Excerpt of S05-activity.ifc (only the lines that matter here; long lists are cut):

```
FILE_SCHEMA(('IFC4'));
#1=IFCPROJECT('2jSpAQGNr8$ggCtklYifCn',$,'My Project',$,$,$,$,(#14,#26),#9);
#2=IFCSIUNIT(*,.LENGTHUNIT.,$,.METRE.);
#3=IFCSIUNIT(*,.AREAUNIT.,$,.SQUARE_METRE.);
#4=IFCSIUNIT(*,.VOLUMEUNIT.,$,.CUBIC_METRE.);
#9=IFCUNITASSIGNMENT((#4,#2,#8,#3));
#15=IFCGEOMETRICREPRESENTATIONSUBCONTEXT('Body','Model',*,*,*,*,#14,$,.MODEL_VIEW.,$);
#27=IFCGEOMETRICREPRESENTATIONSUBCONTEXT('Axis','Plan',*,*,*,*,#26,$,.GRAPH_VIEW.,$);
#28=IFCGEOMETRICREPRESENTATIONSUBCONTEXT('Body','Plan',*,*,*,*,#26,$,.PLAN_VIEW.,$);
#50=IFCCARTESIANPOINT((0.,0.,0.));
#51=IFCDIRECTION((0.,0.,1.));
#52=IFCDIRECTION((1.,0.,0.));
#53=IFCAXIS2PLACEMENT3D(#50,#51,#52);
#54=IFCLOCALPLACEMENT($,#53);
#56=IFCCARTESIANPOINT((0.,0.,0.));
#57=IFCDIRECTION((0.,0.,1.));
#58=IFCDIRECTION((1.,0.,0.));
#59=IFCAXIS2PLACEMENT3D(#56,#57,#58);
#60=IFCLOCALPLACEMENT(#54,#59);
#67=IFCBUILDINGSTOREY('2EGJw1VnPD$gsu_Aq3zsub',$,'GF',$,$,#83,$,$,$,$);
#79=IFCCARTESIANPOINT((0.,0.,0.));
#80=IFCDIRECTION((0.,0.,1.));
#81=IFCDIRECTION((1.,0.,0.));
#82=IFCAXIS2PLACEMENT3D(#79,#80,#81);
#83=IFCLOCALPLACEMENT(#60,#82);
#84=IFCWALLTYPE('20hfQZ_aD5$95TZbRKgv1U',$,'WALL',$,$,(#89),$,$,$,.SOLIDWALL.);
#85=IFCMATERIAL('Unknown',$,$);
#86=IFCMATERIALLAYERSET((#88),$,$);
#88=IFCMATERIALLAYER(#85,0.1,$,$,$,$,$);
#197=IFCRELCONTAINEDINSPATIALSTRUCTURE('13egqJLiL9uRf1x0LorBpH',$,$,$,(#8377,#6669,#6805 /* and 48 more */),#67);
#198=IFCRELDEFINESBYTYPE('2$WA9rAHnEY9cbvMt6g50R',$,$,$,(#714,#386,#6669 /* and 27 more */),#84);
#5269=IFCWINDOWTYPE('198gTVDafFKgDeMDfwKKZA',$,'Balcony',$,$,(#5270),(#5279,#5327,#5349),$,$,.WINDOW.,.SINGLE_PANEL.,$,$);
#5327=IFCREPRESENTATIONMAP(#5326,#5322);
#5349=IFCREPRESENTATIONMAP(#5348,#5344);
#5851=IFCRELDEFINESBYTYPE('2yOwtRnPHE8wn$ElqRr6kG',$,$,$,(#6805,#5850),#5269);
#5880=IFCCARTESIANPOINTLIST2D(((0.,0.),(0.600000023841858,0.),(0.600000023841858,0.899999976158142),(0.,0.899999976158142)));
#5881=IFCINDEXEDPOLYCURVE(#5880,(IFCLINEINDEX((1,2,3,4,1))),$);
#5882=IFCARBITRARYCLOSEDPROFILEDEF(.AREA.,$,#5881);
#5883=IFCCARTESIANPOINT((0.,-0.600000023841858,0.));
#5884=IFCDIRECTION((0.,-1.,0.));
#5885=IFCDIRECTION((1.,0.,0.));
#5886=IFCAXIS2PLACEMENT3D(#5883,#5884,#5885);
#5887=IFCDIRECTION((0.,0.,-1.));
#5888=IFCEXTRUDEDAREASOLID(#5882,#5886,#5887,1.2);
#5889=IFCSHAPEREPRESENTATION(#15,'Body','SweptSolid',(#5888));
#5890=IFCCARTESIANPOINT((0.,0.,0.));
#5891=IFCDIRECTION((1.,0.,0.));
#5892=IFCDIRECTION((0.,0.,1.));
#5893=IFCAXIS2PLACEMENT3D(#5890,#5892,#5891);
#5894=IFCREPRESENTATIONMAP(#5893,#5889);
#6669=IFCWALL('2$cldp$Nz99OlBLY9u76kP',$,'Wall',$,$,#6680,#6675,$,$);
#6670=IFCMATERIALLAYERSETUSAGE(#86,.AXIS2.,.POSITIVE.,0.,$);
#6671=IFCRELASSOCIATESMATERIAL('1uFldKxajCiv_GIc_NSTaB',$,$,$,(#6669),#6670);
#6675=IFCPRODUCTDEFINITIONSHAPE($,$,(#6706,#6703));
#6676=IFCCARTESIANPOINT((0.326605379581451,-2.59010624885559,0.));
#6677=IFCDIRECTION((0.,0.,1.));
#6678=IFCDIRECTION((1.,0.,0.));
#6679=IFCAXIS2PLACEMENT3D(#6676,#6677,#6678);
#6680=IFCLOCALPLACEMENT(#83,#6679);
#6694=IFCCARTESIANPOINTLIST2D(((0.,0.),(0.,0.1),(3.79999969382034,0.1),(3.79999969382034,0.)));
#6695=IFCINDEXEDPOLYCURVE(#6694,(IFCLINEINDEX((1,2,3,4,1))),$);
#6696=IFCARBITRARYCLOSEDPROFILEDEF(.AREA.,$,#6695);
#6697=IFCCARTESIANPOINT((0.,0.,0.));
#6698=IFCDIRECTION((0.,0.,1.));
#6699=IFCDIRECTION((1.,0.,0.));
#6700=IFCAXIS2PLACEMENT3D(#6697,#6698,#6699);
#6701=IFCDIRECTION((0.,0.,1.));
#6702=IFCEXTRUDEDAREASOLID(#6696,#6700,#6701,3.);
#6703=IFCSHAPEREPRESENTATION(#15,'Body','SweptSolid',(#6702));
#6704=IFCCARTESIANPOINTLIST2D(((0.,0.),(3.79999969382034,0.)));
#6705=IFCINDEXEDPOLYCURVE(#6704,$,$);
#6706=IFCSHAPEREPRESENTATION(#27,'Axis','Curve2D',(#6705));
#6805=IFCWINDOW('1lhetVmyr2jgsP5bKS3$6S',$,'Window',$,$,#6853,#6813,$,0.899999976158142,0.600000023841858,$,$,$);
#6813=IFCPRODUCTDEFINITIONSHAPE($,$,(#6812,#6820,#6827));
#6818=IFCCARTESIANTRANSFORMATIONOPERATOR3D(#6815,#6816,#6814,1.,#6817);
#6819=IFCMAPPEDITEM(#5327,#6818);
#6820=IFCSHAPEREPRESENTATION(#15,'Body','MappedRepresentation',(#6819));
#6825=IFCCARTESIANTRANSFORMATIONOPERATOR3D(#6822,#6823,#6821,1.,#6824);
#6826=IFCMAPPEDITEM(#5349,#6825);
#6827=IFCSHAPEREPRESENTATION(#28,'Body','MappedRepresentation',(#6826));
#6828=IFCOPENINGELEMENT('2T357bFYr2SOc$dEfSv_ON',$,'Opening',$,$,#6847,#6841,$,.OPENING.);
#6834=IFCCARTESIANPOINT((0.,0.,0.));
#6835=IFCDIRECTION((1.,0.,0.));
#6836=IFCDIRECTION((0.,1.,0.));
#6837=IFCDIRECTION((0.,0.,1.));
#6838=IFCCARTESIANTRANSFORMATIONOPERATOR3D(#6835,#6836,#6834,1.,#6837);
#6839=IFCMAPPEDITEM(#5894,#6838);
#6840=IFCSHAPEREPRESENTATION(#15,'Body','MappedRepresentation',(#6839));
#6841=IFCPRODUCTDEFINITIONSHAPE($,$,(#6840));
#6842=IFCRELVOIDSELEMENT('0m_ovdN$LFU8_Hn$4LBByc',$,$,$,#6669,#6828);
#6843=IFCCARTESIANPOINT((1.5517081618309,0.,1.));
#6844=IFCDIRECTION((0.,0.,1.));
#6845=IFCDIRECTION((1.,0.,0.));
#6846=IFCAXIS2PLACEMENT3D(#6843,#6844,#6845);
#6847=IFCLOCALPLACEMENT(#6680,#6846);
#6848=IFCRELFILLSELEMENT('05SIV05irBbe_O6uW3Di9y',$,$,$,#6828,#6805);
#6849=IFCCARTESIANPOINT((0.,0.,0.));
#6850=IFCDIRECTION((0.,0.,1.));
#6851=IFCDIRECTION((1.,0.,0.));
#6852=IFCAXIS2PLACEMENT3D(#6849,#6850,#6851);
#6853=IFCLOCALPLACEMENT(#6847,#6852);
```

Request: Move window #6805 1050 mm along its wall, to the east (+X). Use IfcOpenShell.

```python
import ifcopenshell
import ifcopenshell.api.geometry
import ifcopenshell.util.placement

model = ifcopenshell.open("S05-activity.ifc")

window = model.by_guid("1lhetVmyr2jgsP5bKS3$6S")
opening = window.FillsVoids[0].RelatingOpeningElement
wall = opening.VoidsElements[0].RelatingBuildingElement

wall_matrix = ifcopenshell.util.placement.get_local_placement(wall.ObjectPlacement)
shift = wall_matrix[:3, 0] * 1.05
before = ifcopenshell.util.placement.get_local_placement(window.ObjectPlacement)[:3, 3].copy()

# The window is placed relative to its opening, so it follows when the opening moves.
matrix = ifcopenshell.util.placement.get_local_placement(opening.ObjectPlacement)
matrix[:3, 3] += shift
ifcopenshell.api.geometry.edit_object_placement(
    model, product=opening, matrix=matrix, is_si=False, should_transform_children=True
)

after = ifcopenshell.util.placement.get_local_placement(window.ObjectPlacement)[:3, 3]
print("window moved by", (after - before).round(3) + 0.0)

model.write("S05-activity_edited.ifc")
```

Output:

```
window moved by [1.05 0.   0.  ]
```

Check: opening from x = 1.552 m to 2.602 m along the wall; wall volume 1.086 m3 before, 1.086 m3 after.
